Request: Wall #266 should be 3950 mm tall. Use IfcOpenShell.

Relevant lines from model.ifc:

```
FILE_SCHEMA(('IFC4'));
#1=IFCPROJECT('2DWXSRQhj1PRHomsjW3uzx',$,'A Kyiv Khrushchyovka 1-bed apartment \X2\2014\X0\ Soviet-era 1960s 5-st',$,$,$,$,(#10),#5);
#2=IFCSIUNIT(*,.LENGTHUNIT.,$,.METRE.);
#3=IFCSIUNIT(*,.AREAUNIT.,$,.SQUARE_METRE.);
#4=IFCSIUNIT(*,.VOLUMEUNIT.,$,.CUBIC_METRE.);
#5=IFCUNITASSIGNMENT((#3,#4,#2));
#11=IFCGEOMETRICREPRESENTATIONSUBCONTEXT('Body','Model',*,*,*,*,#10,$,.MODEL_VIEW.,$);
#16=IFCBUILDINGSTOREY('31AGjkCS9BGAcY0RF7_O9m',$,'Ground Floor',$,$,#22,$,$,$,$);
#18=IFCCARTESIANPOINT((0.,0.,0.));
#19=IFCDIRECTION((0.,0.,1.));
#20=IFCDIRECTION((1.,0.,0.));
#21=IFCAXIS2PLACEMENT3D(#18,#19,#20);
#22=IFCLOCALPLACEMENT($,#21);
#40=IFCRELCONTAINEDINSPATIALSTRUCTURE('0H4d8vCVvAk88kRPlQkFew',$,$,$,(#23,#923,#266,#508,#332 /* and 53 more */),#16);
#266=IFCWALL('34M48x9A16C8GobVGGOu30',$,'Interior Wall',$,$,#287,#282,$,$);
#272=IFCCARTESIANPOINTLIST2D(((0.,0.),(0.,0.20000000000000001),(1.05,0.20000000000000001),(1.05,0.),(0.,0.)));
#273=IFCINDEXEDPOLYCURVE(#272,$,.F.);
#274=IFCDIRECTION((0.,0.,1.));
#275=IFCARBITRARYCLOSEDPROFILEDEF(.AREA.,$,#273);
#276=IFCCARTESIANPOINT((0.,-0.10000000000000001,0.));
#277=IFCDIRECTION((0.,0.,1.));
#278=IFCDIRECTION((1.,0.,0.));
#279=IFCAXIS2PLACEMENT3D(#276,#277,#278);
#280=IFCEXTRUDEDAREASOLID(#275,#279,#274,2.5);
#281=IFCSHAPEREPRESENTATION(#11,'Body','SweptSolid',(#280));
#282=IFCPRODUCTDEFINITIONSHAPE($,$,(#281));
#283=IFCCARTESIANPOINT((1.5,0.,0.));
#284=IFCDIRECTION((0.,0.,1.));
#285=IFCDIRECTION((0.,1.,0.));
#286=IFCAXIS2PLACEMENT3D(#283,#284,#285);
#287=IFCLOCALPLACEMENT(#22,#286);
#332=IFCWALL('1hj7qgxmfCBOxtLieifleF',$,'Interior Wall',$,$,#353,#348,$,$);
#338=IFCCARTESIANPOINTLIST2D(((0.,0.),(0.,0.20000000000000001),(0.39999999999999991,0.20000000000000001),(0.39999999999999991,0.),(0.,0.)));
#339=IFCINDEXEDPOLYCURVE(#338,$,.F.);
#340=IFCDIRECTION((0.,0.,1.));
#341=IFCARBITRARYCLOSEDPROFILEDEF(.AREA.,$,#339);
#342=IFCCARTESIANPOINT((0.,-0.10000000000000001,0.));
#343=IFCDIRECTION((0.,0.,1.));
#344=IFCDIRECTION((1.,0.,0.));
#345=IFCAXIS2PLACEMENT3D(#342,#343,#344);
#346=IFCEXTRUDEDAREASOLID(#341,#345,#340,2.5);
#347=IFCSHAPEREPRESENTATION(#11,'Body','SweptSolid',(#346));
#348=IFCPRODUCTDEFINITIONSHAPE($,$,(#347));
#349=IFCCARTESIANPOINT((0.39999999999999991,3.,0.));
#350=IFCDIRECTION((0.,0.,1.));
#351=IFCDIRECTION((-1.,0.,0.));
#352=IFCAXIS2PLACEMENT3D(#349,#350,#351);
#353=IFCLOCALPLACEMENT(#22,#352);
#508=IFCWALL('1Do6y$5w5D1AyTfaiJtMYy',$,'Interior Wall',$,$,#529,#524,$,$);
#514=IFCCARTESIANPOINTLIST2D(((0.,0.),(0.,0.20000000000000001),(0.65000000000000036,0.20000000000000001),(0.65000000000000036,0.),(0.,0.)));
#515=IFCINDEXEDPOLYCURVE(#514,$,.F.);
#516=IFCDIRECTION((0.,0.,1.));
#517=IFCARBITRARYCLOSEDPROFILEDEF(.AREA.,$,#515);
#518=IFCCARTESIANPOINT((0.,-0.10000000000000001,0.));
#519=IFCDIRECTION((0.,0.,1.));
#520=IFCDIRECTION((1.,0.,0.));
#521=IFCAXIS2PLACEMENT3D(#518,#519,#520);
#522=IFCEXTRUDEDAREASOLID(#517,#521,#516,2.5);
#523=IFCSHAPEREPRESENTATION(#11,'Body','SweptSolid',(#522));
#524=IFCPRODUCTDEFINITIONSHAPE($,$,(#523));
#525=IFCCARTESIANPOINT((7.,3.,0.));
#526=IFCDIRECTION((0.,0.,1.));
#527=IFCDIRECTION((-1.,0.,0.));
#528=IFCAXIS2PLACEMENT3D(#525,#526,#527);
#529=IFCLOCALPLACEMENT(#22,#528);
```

```python
import ifcopenshell
import ifcopenshell.geom
import ifcopenshell.util.representation
import ifcopenshell.util.shape

model = ifcopenshell.open("model.ifc")
settings = ifcopenshell.geom.settings()


def volume(element):
    """Net volume in cubic metres, openings subtracted."""
    shape = ifcopenshell.geom.create_shape(settings, element)
    return ifcopenshell.util.shape.get_volume(shape.geometry)


wall = model.by_id(266)
before = volume(wall)

body = ifcopenshell.util.representation.get_representation(wall, "Model", "Body")
solid = body.Items[0]
old_height = solid.Depth
solid.Depth = 3.95
after = volume(wall)

print(f"height {old_height:g} -> {solid.Depth:g}, volume {before:.3f} -> {after:.3f} m3")

model.write("model_v2.ifc")
```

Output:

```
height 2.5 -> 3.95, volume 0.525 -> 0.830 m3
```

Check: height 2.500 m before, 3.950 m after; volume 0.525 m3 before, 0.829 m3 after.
